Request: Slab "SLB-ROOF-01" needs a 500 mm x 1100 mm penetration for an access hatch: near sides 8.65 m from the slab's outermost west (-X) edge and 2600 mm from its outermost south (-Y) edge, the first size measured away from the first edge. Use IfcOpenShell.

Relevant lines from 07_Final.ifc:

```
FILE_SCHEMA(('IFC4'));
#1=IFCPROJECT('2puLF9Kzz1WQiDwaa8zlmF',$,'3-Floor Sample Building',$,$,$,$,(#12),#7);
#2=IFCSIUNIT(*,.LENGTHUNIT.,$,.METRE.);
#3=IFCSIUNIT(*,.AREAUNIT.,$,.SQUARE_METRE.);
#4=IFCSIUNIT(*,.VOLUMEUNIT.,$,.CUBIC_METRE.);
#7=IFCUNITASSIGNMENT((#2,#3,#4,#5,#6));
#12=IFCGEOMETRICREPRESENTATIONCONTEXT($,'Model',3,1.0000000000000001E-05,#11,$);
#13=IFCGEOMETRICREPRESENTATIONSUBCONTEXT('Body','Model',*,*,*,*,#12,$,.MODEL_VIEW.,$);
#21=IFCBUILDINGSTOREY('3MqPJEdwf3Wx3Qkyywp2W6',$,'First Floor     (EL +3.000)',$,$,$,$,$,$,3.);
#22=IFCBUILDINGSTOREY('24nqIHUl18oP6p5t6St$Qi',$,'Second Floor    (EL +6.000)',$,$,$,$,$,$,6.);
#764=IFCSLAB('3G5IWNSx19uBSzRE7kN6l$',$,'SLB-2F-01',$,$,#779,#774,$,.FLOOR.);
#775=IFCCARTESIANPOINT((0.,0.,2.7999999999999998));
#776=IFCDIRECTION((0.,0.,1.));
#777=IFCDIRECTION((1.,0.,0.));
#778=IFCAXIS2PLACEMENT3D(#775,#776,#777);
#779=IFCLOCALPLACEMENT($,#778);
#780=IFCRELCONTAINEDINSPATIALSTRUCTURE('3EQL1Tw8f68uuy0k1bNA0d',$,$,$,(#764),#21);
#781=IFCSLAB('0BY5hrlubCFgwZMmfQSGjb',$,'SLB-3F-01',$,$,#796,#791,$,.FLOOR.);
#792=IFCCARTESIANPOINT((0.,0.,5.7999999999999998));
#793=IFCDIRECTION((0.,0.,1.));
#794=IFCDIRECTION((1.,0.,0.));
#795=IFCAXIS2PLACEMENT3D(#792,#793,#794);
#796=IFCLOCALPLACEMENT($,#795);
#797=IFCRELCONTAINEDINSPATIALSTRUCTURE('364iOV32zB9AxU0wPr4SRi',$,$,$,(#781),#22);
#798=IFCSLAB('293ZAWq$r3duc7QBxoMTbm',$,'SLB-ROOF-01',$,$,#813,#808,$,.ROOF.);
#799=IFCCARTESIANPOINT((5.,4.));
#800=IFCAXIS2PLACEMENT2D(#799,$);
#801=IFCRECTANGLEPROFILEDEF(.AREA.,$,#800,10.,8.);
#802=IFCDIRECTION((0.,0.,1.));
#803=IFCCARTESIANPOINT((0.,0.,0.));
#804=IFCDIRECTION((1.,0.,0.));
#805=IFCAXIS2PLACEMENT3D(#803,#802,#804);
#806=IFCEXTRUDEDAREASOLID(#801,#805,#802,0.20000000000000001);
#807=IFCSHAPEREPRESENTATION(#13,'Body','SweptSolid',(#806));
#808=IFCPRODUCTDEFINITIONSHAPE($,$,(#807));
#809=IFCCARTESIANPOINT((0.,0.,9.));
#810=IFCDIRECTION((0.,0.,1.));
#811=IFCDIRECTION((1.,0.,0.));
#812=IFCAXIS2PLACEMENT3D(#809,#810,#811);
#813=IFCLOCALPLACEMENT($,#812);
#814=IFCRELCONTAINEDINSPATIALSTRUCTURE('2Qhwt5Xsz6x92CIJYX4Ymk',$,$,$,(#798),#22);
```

```python
import numpy as np
import ifcopenshell
import ifcopenshell.api.feature
import ifcopenshell.api.geometry
import ifcopenshell.api.root
import ifcopenshell.geom
import ifcopenshell.util.placement
import ifcopenshell.util.representation
import ifcopenshell.util.shape
import ifcopenshell.util.unit

model = ifcopenshell.open("07_Final.ifc")
unit_scale = ifcopenshell.util.unit.calculate_unit_scale(model)
settings = ifcopenshell.geom.settings()


def volume(element):
    """Net volume in cubic metres, openings subtracted."""
    shape = ifcopenshell.geom.create_shape(settings, element)
    return ifcopenshell.util.shape.get_volume(shape.geometry)


slab = model.by_guid("293ZAWq$r3duc7QBxoMTbm")
before = volume(slab)

# Extent in the slab's own axes, in metres. The edges named are its -X and -Y sides.
slab_shape = ifcopenshell.geom.create_shape(settings, slab)
vertices = ifcopenshell.util.shape.get_vertices(slab_shape.geometry)
x_min, y_min, bottom = vertices.min(axis=0)
top = vertices[:, 2].max()

opening = ifcopenshell.api.root.create_entity(model, ifc_class="IfcOpeningElement", name="Access hatch opening", predefined_type="OPENING")
context = ifcopenshell.util.representation.get_context(model, "Model", "Body", "MODEL_VIEW")
width, depth = 0.5, 1.1
outline = [(0.0, 0.0), (width, 0.0), (width, depth), (0.0, depth), (0.0, 0.0)]
# Overshoot both faces by 50 mm so the cut is clean.
shape = ifcopenshell.api.geometry.add_slab_representation(
    model, context=context, depth=top - bottom + 0.1, polyline=outline
)
ifcopenshell.api.geometry.assign_representation(model, product=opening, representation=shape)

matrix = ifcopenshell.util.placement.get_local_placement(slab.ObjectPlacement)
matrix[:, 3] = matrix @ np.append(np.array([x_min + 8.65, y_min + 2.6, bottom - 0.05]) / unit_scale, 1.0)
ifcopenshell.api.geometry.edit_object_placement(model, product=opening, matrix=matrix, is_si=False)
ifcopenshell.api.feature.add_feature(model, feature=opening, element=slab)

after = volume(slab)

print(f"slab volume {before:.3f} -> {after:.3f} m3")

model.write("07_Final_edited.ifc")
```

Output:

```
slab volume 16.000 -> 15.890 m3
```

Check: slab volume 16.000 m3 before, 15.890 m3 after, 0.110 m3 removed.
